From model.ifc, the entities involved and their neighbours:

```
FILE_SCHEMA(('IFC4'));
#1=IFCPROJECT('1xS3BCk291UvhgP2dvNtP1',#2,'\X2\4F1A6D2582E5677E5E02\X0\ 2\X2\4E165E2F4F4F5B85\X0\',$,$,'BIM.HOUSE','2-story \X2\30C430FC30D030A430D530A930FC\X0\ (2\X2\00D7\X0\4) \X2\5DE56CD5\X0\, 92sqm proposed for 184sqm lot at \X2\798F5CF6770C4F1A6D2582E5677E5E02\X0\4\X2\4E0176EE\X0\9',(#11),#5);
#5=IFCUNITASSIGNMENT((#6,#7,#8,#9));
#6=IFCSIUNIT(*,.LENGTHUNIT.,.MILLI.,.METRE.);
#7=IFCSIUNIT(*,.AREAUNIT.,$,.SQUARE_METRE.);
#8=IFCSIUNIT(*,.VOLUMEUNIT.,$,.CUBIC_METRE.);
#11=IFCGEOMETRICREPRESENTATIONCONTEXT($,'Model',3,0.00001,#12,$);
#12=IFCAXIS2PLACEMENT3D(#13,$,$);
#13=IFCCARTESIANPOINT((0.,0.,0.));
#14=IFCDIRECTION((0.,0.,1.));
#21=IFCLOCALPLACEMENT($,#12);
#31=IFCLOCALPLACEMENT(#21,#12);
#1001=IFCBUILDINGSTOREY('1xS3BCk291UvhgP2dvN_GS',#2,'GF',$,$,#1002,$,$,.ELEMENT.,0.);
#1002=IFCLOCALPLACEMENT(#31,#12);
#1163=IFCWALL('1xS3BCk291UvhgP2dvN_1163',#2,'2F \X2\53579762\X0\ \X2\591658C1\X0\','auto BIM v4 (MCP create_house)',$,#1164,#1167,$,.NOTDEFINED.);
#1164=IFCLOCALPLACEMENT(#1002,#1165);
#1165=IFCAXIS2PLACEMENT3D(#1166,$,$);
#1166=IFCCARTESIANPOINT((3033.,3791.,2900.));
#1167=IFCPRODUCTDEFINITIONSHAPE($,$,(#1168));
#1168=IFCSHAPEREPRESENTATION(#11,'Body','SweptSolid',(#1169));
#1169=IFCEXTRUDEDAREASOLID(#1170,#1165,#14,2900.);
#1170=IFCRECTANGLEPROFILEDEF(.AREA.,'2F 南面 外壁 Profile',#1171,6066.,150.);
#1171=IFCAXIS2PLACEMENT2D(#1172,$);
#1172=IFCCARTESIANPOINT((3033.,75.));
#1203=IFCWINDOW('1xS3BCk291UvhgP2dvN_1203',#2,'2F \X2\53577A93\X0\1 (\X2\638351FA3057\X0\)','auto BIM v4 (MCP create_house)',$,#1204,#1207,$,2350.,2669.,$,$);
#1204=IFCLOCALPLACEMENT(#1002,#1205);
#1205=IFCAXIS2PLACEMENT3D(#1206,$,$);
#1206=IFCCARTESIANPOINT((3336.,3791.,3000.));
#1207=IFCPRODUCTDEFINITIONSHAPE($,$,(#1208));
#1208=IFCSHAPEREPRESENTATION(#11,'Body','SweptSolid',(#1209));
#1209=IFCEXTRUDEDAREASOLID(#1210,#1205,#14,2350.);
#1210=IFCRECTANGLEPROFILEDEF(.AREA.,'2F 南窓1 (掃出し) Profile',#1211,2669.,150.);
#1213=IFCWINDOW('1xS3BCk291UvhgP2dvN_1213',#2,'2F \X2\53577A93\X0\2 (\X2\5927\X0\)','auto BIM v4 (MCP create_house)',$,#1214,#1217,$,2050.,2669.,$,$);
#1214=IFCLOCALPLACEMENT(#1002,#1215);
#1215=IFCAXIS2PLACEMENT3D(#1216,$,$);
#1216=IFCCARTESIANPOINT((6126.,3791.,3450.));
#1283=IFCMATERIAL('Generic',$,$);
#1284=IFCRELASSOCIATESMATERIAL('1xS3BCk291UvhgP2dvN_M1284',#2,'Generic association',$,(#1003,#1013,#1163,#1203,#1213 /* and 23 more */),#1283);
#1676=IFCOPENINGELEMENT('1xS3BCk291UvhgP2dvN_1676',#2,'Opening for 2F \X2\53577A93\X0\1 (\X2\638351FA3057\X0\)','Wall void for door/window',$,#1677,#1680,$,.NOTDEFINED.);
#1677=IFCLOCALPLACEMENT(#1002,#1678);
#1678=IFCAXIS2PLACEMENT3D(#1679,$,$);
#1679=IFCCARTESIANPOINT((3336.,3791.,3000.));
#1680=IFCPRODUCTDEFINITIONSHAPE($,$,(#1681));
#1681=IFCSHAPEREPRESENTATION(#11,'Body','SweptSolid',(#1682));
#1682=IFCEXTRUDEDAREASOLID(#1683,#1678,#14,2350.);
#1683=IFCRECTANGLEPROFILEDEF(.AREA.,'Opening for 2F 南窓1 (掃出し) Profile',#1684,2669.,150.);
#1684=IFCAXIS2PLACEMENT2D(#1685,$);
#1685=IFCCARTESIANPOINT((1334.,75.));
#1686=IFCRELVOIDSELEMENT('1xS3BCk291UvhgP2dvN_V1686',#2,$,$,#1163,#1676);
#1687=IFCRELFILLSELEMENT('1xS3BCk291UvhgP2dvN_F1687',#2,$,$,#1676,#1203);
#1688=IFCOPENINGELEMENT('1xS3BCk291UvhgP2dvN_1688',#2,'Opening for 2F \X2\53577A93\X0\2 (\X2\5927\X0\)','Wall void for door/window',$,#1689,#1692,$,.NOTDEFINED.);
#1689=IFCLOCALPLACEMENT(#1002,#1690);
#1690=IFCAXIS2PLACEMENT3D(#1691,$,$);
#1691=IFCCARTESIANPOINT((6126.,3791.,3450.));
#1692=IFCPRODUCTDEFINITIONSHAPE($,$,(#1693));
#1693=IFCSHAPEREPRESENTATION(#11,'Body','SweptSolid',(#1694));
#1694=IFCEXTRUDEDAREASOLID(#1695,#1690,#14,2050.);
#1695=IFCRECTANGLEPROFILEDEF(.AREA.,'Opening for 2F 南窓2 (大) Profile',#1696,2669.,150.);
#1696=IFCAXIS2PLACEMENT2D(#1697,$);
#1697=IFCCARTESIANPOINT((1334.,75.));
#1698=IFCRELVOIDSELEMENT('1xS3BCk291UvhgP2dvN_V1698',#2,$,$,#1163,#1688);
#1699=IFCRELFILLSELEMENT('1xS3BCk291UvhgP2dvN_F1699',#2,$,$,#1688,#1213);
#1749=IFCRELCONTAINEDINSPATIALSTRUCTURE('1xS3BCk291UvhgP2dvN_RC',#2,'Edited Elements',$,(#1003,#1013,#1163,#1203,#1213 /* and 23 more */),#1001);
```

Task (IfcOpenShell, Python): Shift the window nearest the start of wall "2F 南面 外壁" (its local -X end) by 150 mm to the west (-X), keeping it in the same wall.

```python
import ifcopenshell
import ifcopenshell.api.geometry
import ifcopenshell.util.placement

model = ifcopenshell.open("model.ifc")

window = model.by_guid("1xS3BCk291UvhgP2dvN_1203")
opening = window.FillsVoids[0].RelatingOpeningElement
wall = opening.VoidsElements[0].RelatingBuildingElement

wall_matrix = ifcopenshell.util.placement.get_local_placement(wall.ObjectPlacement)
shift = wall_matrix[:3, 0] * -150.0
before = ifcopenshell.util.placement.get_local_placement(window.ObjectPlacement)[:3, 3].copy()

# The window is not placed relative to its opening, so move both.
for product in (opening, window):
    matrix = ifcopenshell.util.placement.get_local_placement(product.ObjectPlacement)
    matrix[:3, 3] += shift
    ifcopenshell.api.geometry.edit_object_placement(model, product=product, matrix=matrix, is_si=False)

after = ifcopenshell.util.placement.get_local_placement(window.ObjectPlacement)[:3, 3]
print("window moved by", (after - before).round(3) + 0.0)

model.write("model_edited.ifc")
```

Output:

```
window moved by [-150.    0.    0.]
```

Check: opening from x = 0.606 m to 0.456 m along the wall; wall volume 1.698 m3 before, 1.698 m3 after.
